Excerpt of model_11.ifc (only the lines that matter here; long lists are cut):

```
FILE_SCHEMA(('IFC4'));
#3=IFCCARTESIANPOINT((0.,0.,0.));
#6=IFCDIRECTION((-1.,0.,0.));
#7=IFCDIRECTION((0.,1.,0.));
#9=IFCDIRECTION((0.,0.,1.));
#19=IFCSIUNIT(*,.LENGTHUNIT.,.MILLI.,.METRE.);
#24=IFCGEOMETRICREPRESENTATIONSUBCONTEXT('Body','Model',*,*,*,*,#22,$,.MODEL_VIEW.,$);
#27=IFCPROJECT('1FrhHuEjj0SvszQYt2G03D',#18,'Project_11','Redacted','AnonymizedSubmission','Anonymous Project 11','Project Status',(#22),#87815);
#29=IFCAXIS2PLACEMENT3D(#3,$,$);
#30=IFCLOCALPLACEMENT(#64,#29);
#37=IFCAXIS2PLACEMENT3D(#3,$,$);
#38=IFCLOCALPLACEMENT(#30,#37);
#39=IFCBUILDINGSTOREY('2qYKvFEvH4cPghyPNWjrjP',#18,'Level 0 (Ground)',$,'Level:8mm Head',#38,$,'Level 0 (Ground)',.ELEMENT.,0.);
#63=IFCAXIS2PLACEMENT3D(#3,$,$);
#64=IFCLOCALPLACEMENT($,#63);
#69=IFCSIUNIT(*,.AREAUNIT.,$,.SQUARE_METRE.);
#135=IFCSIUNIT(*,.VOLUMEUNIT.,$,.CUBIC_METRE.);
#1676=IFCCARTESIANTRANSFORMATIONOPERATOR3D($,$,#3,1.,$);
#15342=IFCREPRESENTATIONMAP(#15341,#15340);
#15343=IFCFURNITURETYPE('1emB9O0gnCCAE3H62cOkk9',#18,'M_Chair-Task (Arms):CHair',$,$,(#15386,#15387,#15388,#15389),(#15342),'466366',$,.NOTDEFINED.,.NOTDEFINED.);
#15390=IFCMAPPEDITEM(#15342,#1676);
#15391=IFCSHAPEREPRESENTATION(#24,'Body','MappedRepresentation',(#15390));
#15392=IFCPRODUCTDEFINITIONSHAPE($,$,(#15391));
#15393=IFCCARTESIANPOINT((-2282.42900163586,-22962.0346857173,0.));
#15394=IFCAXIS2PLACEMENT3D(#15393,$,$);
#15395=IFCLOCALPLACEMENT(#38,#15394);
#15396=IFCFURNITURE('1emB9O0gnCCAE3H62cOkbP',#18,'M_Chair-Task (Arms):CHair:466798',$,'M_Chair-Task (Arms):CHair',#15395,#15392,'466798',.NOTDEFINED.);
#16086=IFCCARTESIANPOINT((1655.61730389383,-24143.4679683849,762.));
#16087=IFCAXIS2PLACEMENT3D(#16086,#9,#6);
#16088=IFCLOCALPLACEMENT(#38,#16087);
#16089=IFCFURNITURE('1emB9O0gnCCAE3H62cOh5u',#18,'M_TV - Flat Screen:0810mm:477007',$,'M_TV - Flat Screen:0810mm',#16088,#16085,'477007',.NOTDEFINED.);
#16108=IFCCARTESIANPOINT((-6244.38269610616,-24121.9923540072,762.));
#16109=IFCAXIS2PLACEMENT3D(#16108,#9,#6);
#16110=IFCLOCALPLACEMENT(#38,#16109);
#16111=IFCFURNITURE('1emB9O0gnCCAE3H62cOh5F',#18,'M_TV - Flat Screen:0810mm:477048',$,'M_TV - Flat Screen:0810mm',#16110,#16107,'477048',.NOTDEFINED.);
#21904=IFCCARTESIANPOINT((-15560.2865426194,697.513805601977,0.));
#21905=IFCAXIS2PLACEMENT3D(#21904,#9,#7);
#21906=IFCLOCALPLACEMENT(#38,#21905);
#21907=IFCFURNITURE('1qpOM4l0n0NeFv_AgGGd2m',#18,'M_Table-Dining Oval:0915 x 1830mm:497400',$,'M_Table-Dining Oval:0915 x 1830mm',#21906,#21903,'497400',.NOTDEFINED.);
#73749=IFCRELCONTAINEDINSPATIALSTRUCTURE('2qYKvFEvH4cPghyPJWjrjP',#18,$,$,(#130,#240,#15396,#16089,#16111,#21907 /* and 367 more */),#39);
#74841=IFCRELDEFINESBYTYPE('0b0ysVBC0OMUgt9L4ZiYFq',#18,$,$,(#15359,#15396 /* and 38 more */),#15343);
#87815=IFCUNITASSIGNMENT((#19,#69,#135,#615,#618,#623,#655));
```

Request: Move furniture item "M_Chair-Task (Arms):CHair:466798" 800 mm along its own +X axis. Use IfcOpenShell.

```python
import ifcopenshell
import ifcopenshell.api.geometry
import ifcopenshell.util.placement

model = ifcopenshell.open("model_11.ifc")

item = model.by_id(15396)
matrix = ifcopenshell.util.placement.get_local_placement(item.ObjectPlacement)
matrix[:3, 3] += matrix[:3, 0] * 800.0
ifcopenshell.api.geometry.edit_object_placement(model, product=item, matrix=matrix, is_si=False)

print(ifcopenshell.util.placement.get_local_placement(item.ObjectPlacement).round(3) + 0.0)

model.write("model_11_v2.ifc")
```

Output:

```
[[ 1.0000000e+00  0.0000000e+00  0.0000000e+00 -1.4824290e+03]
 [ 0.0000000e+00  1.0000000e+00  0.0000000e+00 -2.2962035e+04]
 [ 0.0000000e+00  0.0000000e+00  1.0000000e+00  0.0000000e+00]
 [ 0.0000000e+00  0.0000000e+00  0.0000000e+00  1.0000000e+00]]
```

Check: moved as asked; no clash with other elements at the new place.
